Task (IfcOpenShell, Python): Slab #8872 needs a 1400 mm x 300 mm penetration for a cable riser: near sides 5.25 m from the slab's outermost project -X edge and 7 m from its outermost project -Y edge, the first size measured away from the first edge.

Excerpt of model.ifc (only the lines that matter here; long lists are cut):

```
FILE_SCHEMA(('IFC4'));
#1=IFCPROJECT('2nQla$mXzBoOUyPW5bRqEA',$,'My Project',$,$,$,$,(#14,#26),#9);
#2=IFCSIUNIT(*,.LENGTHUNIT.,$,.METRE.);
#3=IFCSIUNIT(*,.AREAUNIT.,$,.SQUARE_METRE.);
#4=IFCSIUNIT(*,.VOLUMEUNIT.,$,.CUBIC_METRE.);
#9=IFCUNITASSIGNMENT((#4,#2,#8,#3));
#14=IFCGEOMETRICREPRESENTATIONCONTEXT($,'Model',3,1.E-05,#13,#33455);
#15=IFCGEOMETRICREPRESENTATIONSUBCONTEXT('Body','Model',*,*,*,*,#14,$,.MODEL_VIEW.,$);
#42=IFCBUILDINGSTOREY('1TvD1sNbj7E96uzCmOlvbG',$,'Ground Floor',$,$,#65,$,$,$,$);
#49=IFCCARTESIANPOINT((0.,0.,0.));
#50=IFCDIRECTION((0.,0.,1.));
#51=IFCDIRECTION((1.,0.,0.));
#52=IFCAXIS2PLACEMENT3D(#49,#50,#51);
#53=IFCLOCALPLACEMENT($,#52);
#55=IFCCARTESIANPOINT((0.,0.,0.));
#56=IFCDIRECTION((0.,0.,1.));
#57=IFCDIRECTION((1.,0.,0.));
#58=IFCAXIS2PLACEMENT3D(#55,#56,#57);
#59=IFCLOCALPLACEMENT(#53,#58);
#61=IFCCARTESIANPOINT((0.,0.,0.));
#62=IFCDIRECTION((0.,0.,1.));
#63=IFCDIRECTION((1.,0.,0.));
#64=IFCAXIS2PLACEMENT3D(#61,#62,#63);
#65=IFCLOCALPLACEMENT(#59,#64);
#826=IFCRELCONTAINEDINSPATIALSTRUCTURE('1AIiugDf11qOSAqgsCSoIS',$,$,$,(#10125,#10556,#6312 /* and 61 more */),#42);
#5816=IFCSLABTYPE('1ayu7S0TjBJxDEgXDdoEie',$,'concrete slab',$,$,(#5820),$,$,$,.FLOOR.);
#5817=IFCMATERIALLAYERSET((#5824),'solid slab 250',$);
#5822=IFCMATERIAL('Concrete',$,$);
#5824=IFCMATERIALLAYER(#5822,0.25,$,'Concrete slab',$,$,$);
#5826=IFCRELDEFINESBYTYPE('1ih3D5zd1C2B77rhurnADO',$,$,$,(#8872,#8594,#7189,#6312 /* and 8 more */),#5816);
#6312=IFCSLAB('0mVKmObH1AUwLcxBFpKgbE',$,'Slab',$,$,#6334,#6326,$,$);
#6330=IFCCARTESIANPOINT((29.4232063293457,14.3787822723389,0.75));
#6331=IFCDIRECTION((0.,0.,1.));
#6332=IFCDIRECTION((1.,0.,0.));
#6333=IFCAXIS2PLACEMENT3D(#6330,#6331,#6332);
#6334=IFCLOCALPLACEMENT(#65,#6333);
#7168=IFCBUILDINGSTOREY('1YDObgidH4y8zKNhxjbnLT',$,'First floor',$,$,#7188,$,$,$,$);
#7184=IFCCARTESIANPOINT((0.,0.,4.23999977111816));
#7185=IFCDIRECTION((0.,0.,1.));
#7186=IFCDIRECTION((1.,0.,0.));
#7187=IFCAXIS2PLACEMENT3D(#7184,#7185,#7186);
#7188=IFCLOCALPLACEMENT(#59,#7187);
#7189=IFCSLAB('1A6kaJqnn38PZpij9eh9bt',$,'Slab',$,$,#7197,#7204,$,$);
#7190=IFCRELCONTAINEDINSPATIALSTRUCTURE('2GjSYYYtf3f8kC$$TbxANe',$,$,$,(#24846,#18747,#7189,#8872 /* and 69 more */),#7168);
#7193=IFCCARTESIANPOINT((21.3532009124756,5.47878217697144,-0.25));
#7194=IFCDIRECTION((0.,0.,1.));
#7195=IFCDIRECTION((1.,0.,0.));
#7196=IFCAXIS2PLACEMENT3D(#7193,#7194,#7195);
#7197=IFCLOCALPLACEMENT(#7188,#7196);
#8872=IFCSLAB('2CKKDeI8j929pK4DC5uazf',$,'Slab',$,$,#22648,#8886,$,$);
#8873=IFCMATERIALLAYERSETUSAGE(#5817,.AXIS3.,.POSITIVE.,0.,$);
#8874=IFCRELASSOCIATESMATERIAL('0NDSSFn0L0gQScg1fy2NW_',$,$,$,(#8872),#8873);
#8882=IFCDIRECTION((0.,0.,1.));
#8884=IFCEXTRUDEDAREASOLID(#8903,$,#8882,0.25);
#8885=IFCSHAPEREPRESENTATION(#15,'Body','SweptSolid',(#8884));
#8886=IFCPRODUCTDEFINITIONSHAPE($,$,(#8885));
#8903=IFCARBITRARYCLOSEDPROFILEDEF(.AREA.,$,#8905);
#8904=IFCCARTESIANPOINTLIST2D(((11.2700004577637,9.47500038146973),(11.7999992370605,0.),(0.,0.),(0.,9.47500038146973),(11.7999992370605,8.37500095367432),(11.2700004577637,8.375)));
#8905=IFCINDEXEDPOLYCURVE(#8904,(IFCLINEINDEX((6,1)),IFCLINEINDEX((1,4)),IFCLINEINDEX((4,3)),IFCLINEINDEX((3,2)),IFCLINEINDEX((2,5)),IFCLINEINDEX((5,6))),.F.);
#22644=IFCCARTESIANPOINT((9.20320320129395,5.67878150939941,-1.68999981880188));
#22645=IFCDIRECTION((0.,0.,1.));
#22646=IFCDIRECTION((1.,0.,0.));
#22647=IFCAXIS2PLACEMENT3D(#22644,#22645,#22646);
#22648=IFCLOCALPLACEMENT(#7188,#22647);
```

```python
import numpy as np
import ifcopenshell
import ifcopenshell.api.feature
import ifcopenshell.api.geometry
import ifcopenshell.api.root
import ifcopenshell.geom
import ifcopenshell.util.placement
import ifcopenshell.util.representation
import ifcopenshell.util.shape
import ifcopenshell.util.unit

model = ifcopenshell.open("model.ifc")
unit_scale = ifcopenshell.util.unit.calculate_unit_scale(model)
settings = ifcopenshell.geom.settings()


def volume(element):
    """Net volume in cubic metres, openings subtracted."""
    shape = ifcopenshell.geom.create_shape(settings, element)
    return ifcopenshell.util.shape.get_volume(shape.geometry)


slab = model.by_guid("2CKKDeI8j929pK4DC5uazf")
before = volume(slab)

# Extent in the slab's own axes, in metres. The edges named are its -X and -Y sides.
slab_shape = ifcopenshell.geom.create_shape(settings, slab)
vertices = ifcopenshell.util.shape.get_vertices(slab_shape.geometry)
x_min, y_min, bottom = vertices.min(axis=0)
top = vertices[:, 2].max()

opening = ifcopenshell.api.root.create_entity(model, ifc_class="IfcOpeningElement", name="Cable riser opening", predefined_type="OPENING")
context = ifcopenshell.util.representation.get_context(model, "Model", "Body", "MODEL_VIEW")
width, depth = 1.4, 0.3
outline = [(0.0, 0.0), (width, 0.0), (width, depth), (0.0, depth), (0.0, 0.0)]
# Overshoot both faces by 50 mm so the cut is clean.
shape = ifcopenshell.api.geometry.add_slab_representation(
    model, context=context, depth=top - bottom + 0.1, polyline=outline
)
ifcopenshell.api.geometry.assign_representation(model, product=opening, representation=shape)

matrix = ifcopenshell.util.placement.get_local_placement(slab.ObjectPlacement)
matrix[:, 3] = matrix @ np.append(np.array([x_min + 5.25, y_min + 7, bottom - 0.05]) / unit_scale, 1.0)
ifcopenshell.api.geometry.edit_object_placement(model, product=opening, matrix=matrix, is_si=False)
ifcopenshell.api.feature.add_feature(model, feature=opening, element=slab)

after = volume(slab)

print(f"slab volume {before:.3f} -> {after:.3f} m3")

model.write("model_edited.ifc")
```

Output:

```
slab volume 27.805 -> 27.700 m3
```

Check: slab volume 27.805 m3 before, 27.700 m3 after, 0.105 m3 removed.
